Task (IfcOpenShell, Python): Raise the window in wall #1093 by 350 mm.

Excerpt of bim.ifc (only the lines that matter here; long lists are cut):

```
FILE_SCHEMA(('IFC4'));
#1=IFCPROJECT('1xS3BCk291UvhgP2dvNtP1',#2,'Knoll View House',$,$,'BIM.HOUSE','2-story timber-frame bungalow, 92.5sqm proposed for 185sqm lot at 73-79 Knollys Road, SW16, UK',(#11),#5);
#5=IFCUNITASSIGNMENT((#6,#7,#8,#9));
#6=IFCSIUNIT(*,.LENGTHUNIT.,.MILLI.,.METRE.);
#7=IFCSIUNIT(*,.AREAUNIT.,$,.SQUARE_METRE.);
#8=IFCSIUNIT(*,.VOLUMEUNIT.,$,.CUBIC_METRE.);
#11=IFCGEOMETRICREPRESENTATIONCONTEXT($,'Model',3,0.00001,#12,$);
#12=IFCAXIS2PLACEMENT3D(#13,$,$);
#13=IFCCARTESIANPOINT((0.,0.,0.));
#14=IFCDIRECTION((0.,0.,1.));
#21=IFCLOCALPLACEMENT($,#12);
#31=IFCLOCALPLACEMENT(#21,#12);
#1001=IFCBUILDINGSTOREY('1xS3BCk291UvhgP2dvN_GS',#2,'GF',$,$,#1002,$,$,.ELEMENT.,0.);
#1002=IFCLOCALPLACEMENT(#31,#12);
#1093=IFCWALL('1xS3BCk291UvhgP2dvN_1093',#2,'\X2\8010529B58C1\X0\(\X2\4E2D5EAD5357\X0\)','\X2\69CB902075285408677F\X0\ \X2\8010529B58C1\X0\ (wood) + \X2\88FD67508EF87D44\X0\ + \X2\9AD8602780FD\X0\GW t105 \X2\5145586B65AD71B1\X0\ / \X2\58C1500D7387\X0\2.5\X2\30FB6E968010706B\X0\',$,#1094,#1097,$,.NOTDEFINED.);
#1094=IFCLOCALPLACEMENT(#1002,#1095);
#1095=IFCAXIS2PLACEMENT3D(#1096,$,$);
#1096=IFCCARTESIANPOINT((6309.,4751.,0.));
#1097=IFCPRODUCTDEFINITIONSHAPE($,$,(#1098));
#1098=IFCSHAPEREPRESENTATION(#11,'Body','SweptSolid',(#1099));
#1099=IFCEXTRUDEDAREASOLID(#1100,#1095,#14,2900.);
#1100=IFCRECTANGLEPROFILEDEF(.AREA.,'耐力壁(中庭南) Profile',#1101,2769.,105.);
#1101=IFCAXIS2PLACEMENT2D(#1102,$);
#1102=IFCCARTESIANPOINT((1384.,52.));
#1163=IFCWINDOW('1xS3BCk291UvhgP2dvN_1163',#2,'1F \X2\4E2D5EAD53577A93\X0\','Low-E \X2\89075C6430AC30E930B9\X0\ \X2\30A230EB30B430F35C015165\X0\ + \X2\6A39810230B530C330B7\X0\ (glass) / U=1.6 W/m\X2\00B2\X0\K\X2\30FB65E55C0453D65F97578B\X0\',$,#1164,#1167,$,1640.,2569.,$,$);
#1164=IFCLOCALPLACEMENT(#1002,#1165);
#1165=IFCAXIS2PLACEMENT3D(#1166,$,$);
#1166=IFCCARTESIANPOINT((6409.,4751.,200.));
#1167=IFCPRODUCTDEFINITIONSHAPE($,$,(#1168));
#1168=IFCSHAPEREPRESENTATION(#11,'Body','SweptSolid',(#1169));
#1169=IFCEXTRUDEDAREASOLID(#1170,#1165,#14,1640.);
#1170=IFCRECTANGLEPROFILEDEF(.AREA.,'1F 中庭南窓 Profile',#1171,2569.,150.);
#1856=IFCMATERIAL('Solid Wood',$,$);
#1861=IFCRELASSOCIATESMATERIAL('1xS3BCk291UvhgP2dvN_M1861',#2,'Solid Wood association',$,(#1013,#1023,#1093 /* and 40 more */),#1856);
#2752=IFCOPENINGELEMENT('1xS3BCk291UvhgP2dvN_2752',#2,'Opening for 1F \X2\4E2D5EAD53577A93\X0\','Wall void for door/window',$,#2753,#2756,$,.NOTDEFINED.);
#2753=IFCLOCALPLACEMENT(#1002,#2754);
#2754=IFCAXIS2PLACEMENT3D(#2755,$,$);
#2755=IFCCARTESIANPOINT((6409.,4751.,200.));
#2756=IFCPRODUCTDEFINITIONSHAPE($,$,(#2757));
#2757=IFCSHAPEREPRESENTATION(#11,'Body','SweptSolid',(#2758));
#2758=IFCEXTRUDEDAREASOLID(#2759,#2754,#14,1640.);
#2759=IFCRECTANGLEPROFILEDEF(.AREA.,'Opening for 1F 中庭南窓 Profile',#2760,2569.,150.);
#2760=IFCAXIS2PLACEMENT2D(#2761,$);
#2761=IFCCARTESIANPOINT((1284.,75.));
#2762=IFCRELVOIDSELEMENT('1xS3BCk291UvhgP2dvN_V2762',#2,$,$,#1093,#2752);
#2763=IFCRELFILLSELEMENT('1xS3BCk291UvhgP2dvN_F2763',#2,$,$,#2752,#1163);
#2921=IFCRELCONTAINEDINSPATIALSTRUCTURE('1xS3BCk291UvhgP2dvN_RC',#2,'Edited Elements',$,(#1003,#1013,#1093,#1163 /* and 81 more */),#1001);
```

```python
import numpy as np
import ifcopenshell
import ifcopenshell.api.geometry
import ifcopenshell.util.placement
import ifcopenshell.util.unit

model = ifcopenshell.open("bim.ifc")
unit_scale = ifcopenshell.util.unit.calculate_unit_scale(model)

window = model.by_guid("1xS3BCk291UvhgP2dvN_1163")
opening = window.FillsVoids[0].RelatingOpeningElement
dz = 0.35 / unit_scale

shift = np.array([0.0, 0.0, dz])
# The window is not placed relative to its opening, so move both.
for product in (opening, window):
    matrix = ifcopenshell.util.placement.get_local_placement(product.ObjectPlacement)
    matrix[:3, 3] += shift
    ifcopenshell.api.geometry.edit_object_placement(model, product=product, matrix=matrix, is_si=False)

print(f"moved by {dz * unit_scale:+.3f} m")

model.write("bim_rev.ifc")
```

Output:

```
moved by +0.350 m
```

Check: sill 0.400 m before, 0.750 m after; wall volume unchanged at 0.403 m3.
